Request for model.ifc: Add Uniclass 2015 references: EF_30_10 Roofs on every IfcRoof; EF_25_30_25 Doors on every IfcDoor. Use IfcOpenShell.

First a look at what the model holds.

```python
import ifcopenshell

model = ifcopenshell.open("model.ifc")
print(model.schema)
print("classifications:", [c.Name for c in model.by_type("IfcClassification")])
for ifc_class in ("IfcDoor", "IfcRoof", "IfcStair", "IfcWall", "IfcWindow"):
    print(ifc_class, len(model.by_type(ifc_class)))
```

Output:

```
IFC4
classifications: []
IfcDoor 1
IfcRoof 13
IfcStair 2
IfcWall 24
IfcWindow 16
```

```python
import ifcopenshell
import ifcopenshell.api.classification

model = ifcopenshell.open("model.ifc")

system = ifcopenshell.api.classification.add_classification(model, classification="Uniclass 2015")

codes = {
    "IfcRoof": ("EF_30_10", "Roofs"),
    "IfcDoor": ("EF_25_30_25", "Doors"),
}
for ifc_class, (code, name) in codes.items():
    products = model.by_type(ifc_class)
    ifcopenshell.api.classification.add_reference(
        model, products=products, classification=system, identification=code, name=name
    )
    print(code, len(products))

model.write("model_edited.ifc")
```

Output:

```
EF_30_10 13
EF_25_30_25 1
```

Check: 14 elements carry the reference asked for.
